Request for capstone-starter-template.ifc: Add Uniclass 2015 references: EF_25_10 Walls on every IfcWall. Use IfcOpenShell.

First a look at what the model holds.

```python
import ifcopenshell

model = ifcopenshell.open("capstone-starter-template.ifc")
print(model.schema)
print("classifications:", [c.Name for c in model.by_type("IfcClassification")])
for ifc_class in ("IfcDoor", "IfcRoof", "IfcStair", "IfcWall", "IfcWindow"):
    print(ifc_class, len(model.by_type(ifc_class)))
```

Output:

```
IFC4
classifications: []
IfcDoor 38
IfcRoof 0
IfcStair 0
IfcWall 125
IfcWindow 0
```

```python
import ifcopenshell
import ifcopenshell.api.classification

model = ifcopenshell.open("capstone-starter-template.ifc")

system = ifcopenshell.api.classification.add_classification(model, classification="Uniclass 2015")

codes = {
    "IfcWall": ("EF_25_10", "Walls"),
}
for ifc_class, (code, name) in codes.items():
    products = model.by_type(ifc_class)
    ifcopenshell.api.classification.add_reference(
        model, products=products, classification=system, identification=code, name=name
    )
    print(code, len(products))

model.write("capstone-starter-template_v2.ifc")
```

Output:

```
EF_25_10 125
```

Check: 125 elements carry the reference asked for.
